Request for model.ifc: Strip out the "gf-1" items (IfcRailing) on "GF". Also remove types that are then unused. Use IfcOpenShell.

First a look at what the model holds.

```python
import ifcopenshell
import ifcopenshell.util.element

model = ifcopenshell.open("model.ifc")
print(model.schema)
storey = next(s for s in model.by_type("IfcBuildingStorey") if s.Name == "GF")
railings = [e for e in ifcopenshell.util.element.get_decomposition(storey) if e.is_a("IfcRailing")]
seen = {}
for e in railings:
    element_type = ifcopenshell.util.element.get_type(e)
    name = element_type.Name if element_type not in (None, e) else None
    seen[name] = seen.get(name, 0) + 1
for name, count in sorted(seen.items(), key=str):
    print(count, "x", name)
```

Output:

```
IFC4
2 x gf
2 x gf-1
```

```python
import ifcopenshell
import ifcopenshell.api.root
import ifcopenshell.util.element

model = ifcopenshell.open("model.ifc")

storey = next(s for s in model.by_type("IfcBuildingStorey") if s.Name == "GF")
railings = [e for e in ifcopenshell.util.element.get_decomposition(storey) if e.is_a("IfcRailing")]
targets = [e for e in railings if (t := ifcopenshell.util.element.get_type(e)) not in (None, e) and t.Name == "gf-1"]
types = {ifcopenshell.util.element.get_type(e) for e in targets} - {None, *targets}

for e in targets:
    ifcopenshell.api.root.remove_product(model, product=e)
print(len(targets), "removed")

unused = [t for t in types if not ifcopenshell.util.element.get_types(t)]
for t in unused:
    ifcopenshell.api.root.remove_product(model, product=t)
print(len(unused), "unused types removed")

model.write("model_updated.ifc")
```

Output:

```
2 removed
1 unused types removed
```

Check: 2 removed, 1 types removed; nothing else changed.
